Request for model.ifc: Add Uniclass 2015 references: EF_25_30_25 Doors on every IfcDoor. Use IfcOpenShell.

First a look at what the model holds.

```python
import ifcopenshell

model = ifcopenshell.open("model.ifc")
print(model.schema)
print("classifications:", [c.Name for c in model.by_type("IfcClassification")])
for ifc_class in ("IfcDoor", "IfcRoof", "IfcStair", "IfcWall", "IfcWindow"):
    print(ifc_class, len(model.by_type(ifc_class)))
```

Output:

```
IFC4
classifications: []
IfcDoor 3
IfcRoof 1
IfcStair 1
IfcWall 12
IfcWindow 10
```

```python
import ifcopenshell
import ifcopenshell.api.classification

model = ifcopenshell.open("model.ifc")

system = ifcopenshell.api.classification.add_classification(model, classification="Uniclass 2015")

codes = {
    "IfcDoor": ("EF_25_30_25", "Doors"),
}
for ifc_class, (code, name) in codes.items():
    products = model.by_type(ifc_class)
    ifcopenshell.api.classification.add_reference(
        model, products=products, classification=system, identification=code, name=name
    )
    print(code, len(products))

model.write("model_updated.ifc")
```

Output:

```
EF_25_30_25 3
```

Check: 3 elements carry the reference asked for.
